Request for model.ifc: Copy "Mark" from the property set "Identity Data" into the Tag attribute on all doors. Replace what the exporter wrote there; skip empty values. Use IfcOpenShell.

First a look at what the model holds.

```python
import ifcopenshell
import ifcopenshell.util.element

model = ifcopenshell.open("model.ifc")
print(model.schema)
doors = model.by_type("IfcDoor")
print(len(doors), "doors")
for e in doors[:8]:
    source = ifcopenshell.util.element.get_pset(e, "Identity Data", "Mark")
    target = e.Tag
    print(e.id(), repr(source), repr(target), sep=" | ")
```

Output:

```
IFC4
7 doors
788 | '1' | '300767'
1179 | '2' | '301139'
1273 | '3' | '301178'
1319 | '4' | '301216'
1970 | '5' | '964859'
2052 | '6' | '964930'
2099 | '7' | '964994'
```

```python
import ifcopenshell
import ifcopenshell.util.element

model = ifcopenshell.open("model.ifc")

count = 0
for e in model.by_type("IfcDoor"):
    value = ifcopenshell.util.element.get_pset(e, "Identity Data", "Mark")
    current = e.Tag
    if not value or not value.strip() or current == value:
        continue
    e.Tag = value
    count += 1

print(count, "doors updated")

model.write("model_edited.ifc")
```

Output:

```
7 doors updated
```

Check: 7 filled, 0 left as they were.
